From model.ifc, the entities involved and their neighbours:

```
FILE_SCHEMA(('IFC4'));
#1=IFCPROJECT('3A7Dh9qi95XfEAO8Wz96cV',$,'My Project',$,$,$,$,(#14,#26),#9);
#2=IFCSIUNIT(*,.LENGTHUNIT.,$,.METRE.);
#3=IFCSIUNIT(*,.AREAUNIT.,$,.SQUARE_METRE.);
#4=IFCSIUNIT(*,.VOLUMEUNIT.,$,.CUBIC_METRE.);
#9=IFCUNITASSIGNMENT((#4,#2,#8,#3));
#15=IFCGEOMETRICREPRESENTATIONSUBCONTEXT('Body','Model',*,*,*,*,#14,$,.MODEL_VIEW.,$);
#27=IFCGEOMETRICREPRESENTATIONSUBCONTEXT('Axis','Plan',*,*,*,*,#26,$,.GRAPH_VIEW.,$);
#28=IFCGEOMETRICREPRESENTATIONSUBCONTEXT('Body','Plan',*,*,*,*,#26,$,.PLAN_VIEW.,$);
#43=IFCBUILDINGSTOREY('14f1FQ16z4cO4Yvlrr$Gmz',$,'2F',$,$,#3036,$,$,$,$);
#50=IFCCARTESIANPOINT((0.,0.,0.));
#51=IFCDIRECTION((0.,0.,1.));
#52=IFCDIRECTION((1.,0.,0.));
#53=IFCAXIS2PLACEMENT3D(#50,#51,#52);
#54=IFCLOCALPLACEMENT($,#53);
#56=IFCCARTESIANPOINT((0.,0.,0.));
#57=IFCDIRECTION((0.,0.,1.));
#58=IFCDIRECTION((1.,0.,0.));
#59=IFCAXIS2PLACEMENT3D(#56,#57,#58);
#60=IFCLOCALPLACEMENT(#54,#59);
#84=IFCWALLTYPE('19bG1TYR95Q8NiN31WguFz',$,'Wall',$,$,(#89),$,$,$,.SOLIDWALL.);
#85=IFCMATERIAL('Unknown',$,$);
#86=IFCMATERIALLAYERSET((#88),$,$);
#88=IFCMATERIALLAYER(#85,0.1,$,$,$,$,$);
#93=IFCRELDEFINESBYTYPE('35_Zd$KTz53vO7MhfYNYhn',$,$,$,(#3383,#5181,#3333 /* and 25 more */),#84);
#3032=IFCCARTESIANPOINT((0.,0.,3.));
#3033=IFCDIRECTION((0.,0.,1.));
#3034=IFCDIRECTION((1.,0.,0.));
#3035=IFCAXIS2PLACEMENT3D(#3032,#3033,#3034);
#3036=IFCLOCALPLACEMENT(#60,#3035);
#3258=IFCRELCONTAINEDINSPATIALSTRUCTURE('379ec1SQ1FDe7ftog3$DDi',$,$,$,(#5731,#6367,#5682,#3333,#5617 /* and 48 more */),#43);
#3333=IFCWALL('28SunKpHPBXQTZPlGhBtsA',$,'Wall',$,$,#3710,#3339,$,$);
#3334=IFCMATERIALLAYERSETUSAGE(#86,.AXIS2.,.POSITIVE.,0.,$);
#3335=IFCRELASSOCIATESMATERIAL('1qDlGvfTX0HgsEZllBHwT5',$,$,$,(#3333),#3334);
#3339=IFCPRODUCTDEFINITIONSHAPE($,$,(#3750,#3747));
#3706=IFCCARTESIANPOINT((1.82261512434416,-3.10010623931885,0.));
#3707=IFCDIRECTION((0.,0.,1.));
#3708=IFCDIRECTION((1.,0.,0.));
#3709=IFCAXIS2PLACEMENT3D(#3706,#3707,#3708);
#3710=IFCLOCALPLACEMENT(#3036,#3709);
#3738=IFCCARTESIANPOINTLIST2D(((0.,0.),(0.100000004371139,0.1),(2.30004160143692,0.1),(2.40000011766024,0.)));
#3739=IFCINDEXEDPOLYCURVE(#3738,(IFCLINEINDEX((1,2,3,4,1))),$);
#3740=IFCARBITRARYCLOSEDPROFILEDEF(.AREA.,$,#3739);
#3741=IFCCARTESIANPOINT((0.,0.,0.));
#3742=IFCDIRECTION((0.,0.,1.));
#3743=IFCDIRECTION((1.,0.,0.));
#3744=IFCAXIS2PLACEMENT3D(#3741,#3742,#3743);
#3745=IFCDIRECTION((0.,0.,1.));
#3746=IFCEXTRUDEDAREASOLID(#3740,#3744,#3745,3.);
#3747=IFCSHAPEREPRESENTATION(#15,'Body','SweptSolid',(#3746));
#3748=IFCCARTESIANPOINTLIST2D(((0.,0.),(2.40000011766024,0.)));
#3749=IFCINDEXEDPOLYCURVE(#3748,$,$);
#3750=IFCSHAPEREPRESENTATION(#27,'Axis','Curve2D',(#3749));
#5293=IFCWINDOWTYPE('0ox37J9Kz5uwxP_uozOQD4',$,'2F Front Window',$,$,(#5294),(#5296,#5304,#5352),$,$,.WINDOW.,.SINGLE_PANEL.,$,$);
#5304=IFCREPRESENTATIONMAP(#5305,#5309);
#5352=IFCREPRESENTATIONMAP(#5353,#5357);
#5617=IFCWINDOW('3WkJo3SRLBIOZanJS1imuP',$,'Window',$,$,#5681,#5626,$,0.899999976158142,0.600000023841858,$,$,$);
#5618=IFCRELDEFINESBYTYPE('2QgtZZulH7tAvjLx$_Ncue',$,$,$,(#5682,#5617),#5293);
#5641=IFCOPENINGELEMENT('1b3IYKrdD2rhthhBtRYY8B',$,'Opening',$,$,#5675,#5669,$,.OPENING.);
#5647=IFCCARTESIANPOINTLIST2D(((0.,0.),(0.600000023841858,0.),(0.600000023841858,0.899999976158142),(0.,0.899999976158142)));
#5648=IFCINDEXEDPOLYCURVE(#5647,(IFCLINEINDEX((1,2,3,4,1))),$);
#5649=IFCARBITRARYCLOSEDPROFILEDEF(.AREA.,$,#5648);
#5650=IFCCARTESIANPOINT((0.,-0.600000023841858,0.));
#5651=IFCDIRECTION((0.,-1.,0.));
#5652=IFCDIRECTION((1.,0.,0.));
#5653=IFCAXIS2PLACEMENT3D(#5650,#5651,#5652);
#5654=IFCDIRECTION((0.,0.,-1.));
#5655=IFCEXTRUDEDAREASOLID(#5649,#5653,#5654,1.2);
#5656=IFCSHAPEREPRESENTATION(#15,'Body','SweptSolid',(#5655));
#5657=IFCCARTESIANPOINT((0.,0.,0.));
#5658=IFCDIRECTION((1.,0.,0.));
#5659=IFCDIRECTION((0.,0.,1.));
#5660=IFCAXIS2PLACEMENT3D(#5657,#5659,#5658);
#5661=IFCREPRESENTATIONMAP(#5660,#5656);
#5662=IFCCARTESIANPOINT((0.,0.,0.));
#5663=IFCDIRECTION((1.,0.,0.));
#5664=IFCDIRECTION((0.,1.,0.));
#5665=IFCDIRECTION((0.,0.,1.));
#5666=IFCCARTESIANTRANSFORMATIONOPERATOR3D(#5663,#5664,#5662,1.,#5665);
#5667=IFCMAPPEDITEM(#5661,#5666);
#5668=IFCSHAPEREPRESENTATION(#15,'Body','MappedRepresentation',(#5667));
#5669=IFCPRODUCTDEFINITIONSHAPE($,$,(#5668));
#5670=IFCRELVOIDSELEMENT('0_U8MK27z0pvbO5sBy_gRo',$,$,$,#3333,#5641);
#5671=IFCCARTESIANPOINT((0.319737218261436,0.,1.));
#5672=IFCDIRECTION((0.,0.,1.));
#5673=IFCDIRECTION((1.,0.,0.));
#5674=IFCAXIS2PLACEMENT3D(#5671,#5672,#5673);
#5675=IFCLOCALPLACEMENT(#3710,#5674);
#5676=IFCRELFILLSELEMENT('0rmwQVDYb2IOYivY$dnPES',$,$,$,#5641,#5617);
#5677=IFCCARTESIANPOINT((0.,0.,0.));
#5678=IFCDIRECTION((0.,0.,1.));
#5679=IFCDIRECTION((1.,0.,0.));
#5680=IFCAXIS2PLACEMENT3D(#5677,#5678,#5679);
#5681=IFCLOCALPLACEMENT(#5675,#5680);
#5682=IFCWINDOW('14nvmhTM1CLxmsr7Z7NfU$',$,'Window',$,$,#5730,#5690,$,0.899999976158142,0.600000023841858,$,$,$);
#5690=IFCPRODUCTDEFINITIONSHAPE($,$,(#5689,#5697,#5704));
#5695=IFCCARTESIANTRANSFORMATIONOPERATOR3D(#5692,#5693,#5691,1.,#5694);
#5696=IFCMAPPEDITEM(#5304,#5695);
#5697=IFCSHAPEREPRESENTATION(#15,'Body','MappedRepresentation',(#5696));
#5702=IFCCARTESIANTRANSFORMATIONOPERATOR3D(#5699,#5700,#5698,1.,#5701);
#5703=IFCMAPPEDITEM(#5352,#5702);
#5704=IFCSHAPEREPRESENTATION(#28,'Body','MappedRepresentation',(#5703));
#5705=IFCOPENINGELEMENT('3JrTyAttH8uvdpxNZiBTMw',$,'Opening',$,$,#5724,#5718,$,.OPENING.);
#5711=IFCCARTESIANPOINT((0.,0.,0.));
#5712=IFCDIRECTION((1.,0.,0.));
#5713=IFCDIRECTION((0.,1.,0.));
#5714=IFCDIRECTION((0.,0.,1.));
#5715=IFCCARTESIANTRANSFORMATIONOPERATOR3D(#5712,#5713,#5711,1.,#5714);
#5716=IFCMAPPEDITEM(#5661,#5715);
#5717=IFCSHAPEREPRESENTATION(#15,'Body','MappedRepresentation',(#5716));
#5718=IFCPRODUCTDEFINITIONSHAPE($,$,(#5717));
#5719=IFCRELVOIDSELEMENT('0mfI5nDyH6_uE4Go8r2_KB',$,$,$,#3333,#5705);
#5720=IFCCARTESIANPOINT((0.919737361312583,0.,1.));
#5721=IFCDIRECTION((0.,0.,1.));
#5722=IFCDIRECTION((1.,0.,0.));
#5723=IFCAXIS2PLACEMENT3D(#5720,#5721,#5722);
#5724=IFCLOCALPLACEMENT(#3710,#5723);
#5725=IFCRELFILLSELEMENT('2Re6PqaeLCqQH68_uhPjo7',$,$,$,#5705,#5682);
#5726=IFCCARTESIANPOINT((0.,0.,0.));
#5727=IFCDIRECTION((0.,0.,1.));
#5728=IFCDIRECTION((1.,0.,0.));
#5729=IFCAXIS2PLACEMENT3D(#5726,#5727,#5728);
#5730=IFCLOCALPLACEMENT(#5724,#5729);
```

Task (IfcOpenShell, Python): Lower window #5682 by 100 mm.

```python
import numpy as np
import ifcopenshell
import ifcopenshell.api.geometry
import ifcopenshell.util.placement
import ifcopenshell.util.unit

model = ifcopenshell.open("model.ifc")
unit_scale = ifcopenshell.util.unit.calculate_unit_scale(model)

window = model.by_guid("14nvmhTM1CLxmsr7Z7NfU$")
opening = window.FillsVoids[0].RelatingOpeningElement
dz = -0.1

shift = np.array([0.0, 0.0, dz])
# The window is placed relative to its opening, so it follows when the opening moves.
matrix = ifcopenshell.util.placement.get_local_placement(opening.ObjectPlacement)
matrix[:3, 3] += shift
ifcopenshell.api.geometry.edit_object_placement(
    model, product=opening, matrix=matrix, is_si=False, should_transform_children=True
)

print(f"moved by {dz * unit_scale:+.3f} m")

model.write("model_rev.ifc")
```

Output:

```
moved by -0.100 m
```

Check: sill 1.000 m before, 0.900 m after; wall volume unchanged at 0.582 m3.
